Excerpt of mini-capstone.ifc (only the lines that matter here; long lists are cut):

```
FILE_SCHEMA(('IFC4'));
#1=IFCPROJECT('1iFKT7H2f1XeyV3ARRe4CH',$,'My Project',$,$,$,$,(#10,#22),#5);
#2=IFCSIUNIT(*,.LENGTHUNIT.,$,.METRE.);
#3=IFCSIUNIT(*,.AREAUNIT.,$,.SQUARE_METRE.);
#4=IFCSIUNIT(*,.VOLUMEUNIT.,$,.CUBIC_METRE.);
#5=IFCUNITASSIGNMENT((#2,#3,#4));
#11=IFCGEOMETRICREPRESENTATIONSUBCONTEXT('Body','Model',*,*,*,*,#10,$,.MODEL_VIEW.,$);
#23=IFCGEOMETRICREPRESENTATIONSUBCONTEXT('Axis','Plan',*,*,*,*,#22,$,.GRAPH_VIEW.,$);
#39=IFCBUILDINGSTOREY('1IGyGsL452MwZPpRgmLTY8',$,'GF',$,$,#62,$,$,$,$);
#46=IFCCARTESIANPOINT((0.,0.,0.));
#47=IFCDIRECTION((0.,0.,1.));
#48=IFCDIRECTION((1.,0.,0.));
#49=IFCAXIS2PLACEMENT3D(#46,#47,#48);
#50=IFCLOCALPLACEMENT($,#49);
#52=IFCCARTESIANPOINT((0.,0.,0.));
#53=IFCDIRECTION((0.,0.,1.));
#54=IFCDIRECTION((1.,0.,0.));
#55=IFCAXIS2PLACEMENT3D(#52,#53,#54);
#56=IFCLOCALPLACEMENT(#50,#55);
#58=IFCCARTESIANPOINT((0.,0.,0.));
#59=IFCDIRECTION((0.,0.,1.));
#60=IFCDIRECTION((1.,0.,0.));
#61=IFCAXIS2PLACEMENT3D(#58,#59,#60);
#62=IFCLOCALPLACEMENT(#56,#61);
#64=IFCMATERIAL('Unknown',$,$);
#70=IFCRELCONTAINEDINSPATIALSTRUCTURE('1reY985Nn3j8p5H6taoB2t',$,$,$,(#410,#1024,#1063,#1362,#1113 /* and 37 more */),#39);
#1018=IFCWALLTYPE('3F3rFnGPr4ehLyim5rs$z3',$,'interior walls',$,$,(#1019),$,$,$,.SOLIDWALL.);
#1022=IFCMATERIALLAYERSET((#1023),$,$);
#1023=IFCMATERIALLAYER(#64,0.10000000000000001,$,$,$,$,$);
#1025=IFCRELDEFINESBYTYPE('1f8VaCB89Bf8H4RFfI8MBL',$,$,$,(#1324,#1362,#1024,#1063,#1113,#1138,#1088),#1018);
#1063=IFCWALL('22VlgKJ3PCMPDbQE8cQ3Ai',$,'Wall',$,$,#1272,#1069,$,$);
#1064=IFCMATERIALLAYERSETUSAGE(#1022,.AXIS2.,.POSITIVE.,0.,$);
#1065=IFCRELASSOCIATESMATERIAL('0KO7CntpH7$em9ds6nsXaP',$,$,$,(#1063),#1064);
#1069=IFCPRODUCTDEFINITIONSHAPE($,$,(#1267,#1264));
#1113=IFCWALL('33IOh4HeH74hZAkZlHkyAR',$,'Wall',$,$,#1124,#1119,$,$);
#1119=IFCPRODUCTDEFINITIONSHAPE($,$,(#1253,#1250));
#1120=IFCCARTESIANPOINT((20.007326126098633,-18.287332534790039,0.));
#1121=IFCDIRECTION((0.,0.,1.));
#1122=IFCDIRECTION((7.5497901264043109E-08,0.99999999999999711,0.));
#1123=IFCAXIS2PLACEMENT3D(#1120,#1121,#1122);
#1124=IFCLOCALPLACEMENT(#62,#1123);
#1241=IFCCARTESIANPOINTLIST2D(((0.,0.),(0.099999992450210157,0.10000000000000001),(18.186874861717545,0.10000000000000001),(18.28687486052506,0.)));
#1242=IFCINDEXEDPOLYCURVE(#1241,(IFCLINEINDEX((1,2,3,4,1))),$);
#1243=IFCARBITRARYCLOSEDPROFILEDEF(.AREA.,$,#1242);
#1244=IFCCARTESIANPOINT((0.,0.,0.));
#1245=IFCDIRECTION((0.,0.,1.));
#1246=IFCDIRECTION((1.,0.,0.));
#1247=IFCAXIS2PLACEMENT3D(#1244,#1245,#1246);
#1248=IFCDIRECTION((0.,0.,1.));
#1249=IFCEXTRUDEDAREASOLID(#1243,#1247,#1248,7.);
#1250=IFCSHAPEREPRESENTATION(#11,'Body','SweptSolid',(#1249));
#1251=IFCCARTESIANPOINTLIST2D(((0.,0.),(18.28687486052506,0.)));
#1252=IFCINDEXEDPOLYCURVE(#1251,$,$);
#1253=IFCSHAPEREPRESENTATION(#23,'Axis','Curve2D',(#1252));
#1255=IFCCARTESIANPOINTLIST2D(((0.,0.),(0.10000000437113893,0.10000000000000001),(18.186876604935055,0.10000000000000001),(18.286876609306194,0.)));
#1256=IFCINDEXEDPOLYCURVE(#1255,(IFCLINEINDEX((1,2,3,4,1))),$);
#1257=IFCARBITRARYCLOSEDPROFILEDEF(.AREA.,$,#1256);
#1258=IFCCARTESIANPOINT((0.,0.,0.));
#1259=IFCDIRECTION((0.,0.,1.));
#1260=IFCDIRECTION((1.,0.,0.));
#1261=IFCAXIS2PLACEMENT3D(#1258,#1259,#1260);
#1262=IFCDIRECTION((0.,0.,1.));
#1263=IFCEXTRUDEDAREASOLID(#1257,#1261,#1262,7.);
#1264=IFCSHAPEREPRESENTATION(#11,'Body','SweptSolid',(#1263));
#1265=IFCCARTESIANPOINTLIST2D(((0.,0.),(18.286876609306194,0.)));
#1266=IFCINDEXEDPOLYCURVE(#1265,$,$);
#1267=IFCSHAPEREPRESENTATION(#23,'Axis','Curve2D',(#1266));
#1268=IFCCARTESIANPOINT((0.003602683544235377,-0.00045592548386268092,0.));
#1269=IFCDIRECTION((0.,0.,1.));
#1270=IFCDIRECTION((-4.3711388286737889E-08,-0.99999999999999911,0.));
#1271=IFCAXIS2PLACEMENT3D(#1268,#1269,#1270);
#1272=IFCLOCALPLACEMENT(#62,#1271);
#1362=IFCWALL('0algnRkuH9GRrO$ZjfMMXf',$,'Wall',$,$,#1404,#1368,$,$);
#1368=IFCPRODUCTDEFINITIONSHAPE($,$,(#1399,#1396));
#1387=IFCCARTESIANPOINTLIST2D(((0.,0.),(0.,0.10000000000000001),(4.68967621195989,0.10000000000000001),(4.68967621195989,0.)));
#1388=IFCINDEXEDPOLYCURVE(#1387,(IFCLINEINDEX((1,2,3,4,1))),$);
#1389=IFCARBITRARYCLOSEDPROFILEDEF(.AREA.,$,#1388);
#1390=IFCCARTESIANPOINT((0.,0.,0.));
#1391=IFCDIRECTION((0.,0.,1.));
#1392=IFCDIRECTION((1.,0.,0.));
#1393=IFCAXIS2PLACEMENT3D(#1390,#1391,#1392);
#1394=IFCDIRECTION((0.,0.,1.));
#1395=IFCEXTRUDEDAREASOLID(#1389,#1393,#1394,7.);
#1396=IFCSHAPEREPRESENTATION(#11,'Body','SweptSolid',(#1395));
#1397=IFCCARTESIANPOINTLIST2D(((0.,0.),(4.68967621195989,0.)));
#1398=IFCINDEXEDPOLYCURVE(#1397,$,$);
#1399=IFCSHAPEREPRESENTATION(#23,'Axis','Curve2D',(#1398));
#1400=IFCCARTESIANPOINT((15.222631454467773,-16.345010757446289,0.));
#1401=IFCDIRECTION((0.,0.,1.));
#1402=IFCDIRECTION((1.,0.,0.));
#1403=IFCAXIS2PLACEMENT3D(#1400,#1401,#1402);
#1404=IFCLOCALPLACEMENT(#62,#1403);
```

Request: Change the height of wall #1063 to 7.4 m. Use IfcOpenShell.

```python
import ifcopenshell
import ifcopenshell.geom
import ifcopenshell.util.representation
import ifcopenshell.util.shape

model = ifcopenshell.open("mini-capstone.ifc")
settings = ifcopenshell.geom.settings()


def volume(element):
    """Net volume in cubic metres, openings subtracted."""
    shape = ifcopenshell.geom.create_shape(settings, element)
    return ifcopenshell.util.shape.get_volume(shape.geometry)


wall = model.by_id(1063)
before = volume(wall)

body = ifcopenshell.util.representation.get_representation(wall, "Model", "Body")
solid = body.Items[0]
old_height = solid.Depth
solid.Depth = 7.4
after = volume(wall)

print(f"height {old_height:g} -> {solid.Depth:g}, volume {before:.3f} -> {after:.3f} m3")

model.write("mini-capstone_rev.ifc")
```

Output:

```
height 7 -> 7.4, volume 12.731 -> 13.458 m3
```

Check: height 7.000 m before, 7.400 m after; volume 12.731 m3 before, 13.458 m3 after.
